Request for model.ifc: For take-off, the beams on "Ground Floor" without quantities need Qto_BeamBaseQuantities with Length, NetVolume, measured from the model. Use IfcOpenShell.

First a look at what the model holds.

```python
import ifcopenshell
import ifcopenshell.util.element
import ifcopenshell.util.unit

model = ifcopenshell.open("model.ifc")
print(model.schema)
for unit_type in ("LENGTHUNIT", "AREAUNIT", "VOLUMEUNIT"):
    print(unit_type, ifcopenshell.util.unit.calculate_unit_scale(model, unit_type))
storey = next(s for s in model.by_type("IfcBuildingStorey") if s.Name == "Ground Floor")
beams = [e for e in ifcopenshell.util.element.get_decomposition(storey) if e.is_a("IfcBeam")]
for e in sorted(beams, key=lambda e: e.id()):
    print(e.id(), e.is_a(), e.Name, list(ifcopenshell.util.element.get_psets(e, qtos_only=True)), sep=" | ")
```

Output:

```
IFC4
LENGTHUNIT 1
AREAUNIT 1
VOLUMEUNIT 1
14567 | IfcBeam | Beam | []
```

```python
import ifcopenshell
import ifcopenshell.api.pset
import ifcopenshell.geom
import ifcopenshell.util.element
import ifcopenshell.util.shape
import ifcopenshell.util.unit

model = ifcopenshell.open("model.ifc")
unit_scale = ifcopenshell.util.unit.calculate_unit_scale(model)
volume_scale = ifcopenshell.util.unit.calculate_unit_scale(model, "VOLUMEUNIT")
settings = ifcopenshell.geom.settings()

storey = next(s for s in model.by_type("IfcBuildingStorey") if s.Name == "Ground Floor")
beams = [e for e in ifcopenshell.util.element.get_decomposition(storey) if e.is_a("IfcBeam")]

for e in sorted(beams, key=lambda e: e.id()):
    if ifcopenshell.util.element.get_psets(e, qtos_only=True, should_inherit=False):
        continue
    # Geometry comes back in metres, in the element's own axes.
    shape = ifcopenshell.geom.create_shape(settings, e)
    values = {
        "Length": ifcopenshell.util.shape.get_max_xyz(shape.geometry) / unit_scale,
        "NetVolume": ifcopenshell.util.shape.get_volume(shape.geometry) / volume_scale,
    }
    qto = ifcopenshell.api.pset.add_qto(model, product=e, name="Qto_BeamBaseQuantities")
    ifcopenshell.api.pset.edit_qto(model, qto=qto, properties=values)
    print(e.id(), {k: round(v, 3) for k, v in values.items()})

model.write("model_updated.ifc")
```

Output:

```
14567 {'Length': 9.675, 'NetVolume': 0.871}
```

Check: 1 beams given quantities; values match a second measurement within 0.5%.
